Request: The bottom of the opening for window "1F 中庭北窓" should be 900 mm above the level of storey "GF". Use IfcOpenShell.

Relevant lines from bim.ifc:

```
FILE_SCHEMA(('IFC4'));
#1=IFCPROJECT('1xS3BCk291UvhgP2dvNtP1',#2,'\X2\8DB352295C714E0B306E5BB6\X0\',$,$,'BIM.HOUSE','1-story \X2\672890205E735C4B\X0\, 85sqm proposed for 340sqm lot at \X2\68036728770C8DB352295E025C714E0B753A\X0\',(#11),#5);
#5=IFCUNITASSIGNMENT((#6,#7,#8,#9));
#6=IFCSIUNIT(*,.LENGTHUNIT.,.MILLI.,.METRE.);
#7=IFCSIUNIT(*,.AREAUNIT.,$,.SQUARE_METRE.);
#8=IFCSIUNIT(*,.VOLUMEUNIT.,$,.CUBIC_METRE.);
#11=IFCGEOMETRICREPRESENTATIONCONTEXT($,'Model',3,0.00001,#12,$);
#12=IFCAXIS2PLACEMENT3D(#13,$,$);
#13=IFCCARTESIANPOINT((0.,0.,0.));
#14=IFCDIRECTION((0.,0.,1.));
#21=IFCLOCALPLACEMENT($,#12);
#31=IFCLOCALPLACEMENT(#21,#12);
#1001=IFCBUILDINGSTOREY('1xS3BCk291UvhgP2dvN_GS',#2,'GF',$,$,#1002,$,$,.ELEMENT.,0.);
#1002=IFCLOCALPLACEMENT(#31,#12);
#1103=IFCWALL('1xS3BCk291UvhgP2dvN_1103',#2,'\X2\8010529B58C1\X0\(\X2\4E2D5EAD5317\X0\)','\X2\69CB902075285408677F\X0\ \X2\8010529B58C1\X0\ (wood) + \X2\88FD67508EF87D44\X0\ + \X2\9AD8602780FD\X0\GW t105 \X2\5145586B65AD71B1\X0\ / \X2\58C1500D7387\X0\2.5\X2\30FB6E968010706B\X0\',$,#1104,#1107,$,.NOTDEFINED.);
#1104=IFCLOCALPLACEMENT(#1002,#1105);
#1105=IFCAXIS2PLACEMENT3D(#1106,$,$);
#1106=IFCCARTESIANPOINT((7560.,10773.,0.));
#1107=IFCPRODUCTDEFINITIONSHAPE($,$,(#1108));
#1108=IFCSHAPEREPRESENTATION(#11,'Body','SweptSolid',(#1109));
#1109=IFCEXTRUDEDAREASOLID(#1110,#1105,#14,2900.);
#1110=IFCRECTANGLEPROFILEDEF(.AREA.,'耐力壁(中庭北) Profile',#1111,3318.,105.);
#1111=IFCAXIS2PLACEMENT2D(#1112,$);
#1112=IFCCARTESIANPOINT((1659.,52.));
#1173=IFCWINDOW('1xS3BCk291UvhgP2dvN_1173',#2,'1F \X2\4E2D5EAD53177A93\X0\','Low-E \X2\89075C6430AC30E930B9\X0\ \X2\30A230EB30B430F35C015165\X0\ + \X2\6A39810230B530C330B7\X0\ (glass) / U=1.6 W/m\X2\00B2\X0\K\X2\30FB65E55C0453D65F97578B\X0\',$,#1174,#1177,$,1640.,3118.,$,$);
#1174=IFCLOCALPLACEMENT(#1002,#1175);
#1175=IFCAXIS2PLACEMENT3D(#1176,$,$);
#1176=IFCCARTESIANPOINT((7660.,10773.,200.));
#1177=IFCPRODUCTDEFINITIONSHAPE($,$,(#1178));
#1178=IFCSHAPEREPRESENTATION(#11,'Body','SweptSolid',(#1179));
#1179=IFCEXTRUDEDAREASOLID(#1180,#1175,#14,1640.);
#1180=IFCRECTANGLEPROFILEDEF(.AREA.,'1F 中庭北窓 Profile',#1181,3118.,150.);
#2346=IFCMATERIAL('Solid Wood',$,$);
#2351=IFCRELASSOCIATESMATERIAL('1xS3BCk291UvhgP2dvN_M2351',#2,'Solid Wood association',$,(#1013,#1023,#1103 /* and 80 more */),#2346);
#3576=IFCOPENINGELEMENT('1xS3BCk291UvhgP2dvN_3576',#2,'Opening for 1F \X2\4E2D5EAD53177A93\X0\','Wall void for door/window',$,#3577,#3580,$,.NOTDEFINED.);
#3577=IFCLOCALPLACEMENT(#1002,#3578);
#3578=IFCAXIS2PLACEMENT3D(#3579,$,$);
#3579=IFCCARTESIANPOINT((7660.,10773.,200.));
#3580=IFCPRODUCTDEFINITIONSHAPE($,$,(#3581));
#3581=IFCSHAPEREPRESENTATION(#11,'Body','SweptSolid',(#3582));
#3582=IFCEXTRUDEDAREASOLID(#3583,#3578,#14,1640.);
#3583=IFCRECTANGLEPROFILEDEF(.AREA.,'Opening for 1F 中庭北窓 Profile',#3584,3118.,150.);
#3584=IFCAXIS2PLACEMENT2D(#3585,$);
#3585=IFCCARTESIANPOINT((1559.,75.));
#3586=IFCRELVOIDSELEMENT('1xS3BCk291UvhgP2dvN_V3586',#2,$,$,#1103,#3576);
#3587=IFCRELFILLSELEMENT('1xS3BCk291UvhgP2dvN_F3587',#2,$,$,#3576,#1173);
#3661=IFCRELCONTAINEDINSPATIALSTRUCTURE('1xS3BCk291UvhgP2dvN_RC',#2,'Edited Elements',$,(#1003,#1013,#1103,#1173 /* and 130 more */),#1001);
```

```python
import numpy as np
import ifcopenshell
import ifcopenshell.api.geometry
import ifcopenshell.geom
import ifcopenshell.util.element
import ifcopenshell.util.placement
import ifcopenshell.util.shape
import ifcopenshell.util.unit

model = ifcopenshell.open("bim.ifc")
unit_scale = ifcopenshell.util.unit.calculate_unit_scale(model)

window = model.by_id(1173)
opening = window.FillsVoids[0].RelatingOpeningElement
storey = ifcopenshell.util.element.get_container(window, ifc_class="IfcBuildingStorey")
level = ifcopenshell.util.placement.get_local_placement(storey.ObjectPlacement)[2, 3]

# The opening's origin need not be at the sill, so measure its lowest point.
shape = ifcopenshell.geom.create_shape(ifcopenshell.geom.settings(), opening)
bottom = ifcopenshell.util.shape.get_shape_bottom_elevation(shape, shape.geometry) / unit_scale
dz = level + 0.9 / unit_scale - bottom

shift = np.array([0.0, 0.0, dz])
# The window is not placed relative to its opening, so move both.
for product in (opening, window):
    matrix = ifcopenshell.util.placement.get_local_placement(product.ObjectPlacement)
    matrix[:3, 3] += shift
    ifcopenshell.api.geometry.edit_object_placement(model, product=product, matrix=matrix, is_si=False)

print(f"moved by {dz * unit_scale:+.3f} m")

model.write("bim-out.ifc")
```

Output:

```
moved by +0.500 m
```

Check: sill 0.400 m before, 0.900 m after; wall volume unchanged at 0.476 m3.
